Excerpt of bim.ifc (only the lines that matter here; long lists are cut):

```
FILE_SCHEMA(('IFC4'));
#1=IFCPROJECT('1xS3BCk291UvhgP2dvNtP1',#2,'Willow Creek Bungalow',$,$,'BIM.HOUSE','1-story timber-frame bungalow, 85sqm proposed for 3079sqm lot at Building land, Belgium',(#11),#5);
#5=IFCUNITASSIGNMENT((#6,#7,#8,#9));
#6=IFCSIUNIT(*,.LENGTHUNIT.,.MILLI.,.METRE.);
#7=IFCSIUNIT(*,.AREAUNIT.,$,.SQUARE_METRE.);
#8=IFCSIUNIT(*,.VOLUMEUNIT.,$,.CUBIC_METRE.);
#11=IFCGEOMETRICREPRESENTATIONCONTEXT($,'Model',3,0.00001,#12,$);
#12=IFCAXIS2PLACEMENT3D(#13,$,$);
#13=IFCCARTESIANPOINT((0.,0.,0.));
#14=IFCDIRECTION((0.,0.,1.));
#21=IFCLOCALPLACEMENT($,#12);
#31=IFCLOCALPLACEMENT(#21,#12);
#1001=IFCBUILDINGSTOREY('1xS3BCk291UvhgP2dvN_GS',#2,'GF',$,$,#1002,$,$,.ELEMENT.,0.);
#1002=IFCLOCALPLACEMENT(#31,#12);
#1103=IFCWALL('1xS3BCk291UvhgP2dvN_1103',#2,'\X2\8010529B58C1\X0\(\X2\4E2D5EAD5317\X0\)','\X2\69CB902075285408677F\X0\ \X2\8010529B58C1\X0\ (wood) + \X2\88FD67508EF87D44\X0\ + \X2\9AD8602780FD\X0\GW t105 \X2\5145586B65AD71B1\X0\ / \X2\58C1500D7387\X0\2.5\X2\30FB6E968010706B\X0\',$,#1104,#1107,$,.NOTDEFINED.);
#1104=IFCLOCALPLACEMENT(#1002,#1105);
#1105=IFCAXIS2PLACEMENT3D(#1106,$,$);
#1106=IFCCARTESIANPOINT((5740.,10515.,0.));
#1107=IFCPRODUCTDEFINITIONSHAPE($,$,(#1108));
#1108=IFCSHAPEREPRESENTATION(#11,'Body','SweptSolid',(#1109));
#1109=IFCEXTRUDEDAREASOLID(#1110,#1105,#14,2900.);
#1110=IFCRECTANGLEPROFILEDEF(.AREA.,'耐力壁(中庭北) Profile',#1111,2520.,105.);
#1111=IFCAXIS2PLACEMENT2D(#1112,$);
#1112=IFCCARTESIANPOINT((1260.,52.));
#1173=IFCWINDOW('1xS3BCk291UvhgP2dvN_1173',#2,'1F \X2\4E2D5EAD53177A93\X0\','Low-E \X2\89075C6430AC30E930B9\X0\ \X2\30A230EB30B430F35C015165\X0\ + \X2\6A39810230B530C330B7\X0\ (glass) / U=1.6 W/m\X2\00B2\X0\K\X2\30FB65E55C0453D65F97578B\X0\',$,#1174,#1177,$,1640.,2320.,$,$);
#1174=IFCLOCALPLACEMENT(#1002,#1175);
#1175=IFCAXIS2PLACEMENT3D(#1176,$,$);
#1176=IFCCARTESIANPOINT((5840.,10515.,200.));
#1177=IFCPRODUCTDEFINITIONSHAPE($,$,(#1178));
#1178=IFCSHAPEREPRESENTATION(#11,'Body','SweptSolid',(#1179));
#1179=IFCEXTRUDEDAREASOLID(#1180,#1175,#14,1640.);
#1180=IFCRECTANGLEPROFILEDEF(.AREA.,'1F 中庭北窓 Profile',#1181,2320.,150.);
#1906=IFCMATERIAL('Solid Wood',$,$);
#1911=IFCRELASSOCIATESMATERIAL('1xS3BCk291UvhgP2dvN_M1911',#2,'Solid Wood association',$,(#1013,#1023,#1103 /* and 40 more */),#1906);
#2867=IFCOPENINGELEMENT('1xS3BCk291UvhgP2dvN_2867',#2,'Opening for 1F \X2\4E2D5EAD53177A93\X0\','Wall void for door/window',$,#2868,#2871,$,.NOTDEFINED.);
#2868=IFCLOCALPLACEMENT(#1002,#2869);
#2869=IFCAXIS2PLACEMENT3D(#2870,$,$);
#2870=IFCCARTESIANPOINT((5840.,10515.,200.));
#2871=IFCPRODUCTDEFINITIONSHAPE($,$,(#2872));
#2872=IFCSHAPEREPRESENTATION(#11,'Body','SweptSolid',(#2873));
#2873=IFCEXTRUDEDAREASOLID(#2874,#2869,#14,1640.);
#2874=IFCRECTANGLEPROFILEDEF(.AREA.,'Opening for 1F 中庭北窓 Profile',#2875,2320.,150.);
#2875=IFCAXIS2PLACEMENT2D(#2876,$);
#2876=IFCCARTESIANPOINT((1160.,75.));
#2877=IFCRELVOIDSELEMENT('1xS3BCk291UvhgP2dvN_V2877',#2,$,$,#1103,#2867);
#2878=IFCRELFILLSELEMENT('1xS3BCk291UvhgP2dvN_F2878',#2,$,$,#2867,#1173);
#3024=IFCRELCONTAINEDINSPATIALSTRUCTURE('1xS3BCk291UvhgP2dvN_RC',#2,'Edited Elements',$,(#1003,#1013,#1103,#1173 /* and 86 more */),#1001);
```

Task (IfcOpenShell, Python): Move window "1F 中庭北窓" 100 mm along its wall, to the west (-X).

```python
import ifcopenshell
import ifcopenshell.api.geometry
import ifcopenshell.util.placement
import ifcopenshell.util.unit

model = ifcopenshell.open("bim.ifc")
unit_scale = ifcopenshell.util.unit.calculate_unit_scale(model)

window = model.by_guid("1xS3BCk291UvhgP2dvN_1173")
opening = window.FillsVoids[0].RelatingOpeningElement
wall = opening.VoidsElements[0].RelatingBuildingElement

wall_matrix = ifcopenshell.util.placement.get_local_placement(wall.ObjectPlacement)
shift = wall_matrix[:3, 0] * -0.1 / unit_scale
before = ifcopenshell.util.placement.get_local_placement(window.ObjectPlacement)[:3, 3].copy()

# The window is not placed relative to its opening, so move both.
for product in (opening, window):
    matrix = ifcopenshell.util.placement.get_local_placement(product.ObjectPlacement)
    matrix[:3, 3] += shift
    ifcopenshell.api.geometry.edit_object_placement(model, product=product, matrix=matrix, is_si=False)

after = ifcopenshell.util.placement.get_local_placement(window.ObjectPlacement)[:3, 3]
print("window moved by", (after - before).round(3) + 0.0)

model.write("bim_v2.ifc")
```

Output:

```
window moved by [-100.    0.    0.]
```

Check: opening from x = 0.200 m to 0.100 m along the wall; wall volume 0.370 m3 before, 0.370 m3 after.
